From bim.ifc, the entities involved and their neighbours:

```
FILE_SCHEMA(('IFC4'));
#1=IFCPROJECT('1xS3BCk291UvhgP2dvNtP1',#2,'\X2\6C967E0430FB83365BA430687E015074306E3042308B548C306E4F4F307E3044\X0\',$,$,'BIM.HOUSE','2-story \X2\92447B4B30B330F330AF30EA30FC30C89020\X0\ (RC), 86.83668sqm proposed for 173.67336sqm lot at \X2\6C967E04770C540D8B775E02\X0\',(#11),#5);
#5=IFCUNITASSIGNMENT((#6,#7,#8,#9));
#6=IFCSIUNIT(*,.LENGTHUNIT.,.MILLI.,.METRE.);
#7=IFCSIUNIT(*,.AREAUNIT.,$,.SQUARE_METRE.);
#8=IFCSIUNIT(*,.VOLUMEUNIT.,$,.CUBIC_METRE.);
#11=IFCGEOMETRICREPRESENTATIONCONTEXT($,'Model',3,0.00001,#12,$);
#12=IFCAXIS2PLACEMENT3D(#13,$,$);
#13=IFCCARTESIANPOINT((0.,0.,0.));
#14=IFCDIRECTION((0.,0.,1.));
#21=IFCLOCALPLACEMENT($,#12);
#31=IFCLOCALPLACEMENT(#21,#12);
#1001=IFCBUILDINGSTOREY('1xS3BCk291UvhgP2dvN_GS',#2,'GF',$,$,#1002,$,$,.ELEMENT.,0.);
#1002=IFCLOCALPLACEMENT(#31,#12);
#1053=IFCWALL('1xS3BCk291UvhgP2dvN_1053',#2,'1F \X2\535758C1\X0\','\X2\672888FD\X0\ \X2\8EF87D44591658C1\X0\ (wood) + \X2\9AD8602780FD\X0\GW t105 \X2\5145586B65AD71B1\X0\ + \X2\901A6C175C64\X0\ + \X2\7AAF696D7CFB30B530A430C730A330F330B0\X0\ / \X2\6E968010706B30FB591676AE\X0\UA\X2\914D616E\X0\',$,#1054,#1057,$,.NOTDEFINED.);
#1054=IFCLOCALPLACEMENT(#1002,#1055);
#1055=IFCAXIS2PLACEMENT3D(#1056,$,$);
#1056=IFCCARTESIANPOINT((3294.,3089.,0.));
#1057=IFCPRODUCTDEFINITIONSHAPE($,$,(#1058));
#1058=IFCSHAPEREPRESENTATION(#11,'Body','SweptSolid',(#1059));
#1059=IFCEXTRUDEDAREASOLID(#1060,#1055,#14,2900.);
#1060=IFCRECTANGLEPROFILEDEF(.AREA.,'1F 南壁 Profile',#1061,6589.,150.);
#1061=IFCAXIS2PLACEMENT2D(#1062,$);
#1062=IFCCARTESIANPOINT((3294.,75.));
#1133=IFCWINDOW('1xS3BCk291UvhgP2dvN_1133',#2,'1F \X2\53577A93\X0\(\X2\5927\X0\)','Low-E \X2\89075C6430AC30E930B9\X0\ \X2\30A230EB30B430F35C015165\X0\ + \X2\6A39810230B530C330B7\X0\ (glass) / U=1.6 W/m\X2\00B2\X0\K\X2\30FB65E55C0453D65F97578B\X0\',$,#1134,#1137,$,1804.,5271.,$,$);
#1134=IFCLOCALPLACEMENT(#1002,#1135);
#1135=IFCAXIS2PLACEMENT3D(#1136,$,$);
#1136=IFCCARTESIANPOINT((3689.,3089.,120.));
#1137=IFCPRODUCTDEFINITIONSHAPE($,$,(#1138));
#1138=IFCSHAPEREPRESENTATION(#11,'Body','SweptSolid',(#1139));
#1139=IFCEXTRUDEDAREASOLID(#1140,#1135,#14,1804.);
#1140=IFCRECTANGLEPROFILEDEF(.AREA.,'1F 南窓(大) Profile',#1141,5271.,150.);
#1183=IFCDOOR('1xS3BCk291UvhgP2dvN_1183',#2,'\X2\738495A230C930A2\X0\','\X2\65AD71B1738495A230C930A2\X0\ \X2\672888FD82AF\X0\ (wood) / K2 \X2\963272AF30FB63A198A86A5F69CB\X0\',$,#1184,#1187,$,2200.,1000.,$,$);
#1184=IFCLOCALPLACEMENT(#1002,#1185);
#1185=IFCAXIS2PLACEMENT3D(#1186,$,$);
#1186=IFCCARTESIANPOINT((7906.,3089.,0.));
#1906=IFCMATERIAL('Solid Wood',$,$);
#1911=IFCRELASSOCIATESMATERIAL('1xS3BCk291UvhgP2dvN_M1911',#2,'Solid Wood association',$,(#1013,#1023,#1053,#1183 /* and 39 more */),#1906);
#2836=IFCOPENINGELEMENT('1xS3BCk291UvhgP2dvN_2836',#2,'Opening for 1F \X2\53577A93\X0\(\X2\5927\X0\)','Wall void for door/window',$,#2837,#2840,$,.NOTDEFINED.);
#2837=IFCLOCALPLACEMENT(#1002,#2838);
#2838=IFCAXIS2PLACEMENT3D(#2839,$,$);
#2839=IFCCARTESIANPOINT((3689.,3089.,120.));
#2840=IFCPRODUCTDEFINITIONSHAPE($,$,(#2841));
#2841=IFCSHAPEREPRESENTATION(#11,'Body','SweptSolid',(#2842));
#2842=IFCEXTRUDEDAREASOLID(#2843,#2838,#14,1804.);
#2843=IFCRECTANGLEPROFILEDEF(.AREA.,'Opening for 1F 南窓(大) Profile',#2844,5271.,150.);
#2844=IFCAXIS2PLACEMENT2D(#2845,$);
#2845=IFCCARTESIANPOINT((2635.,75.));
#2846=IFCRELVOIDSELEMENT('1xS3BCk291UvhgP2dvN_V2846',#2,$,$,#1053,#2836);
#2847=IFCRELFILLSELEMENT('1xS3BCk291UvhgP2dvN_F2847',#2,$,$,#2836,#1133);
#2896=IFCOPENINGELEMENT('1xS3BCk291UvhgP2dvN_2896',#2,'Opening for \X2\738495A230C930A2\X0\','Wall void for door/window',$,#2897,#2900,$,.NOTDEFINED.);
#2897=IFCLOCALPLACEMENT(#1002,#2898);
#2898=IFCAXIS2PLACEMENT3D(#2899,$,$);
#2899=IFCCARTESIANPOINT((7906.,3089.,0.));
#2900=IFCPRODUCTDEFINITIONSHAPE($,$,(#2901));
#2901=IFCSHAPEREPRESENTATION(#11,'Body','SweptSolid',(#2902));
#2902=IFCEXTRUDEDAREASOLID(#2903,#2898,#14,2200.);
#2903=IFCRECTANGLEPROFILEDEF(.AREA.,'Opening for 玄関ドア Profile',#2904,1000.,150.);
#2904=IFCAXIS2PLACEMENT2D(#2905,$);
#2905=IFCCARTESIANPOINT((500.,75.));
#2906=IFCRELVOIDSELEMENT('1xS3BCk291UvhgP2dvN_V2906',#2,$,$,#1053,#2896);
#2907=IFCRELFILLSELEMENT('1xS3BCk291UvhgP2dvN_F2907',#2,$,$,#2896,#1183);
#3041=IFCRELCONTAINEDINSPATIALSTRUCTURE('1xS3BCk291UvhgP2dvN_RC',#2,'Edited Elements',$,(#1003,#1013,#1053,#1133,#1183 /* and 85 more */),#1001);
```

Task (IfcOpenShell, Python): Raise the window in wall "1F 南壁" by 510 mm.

```python
import numpy as np
import ifcopenshell
import ifcopenshell.api.geometry
import ifcopenshell.util.placement
import ifcopenshell.util.unit

model = ifcopenshell.open("bim.ifc")
unit_scale = ifcopenshell.util.unit.calculate_unit_scale(model)

window = model.by_guid("1xS3BCk291UvhgP2dvN_1133")
opening = window.FillsVoids[0].RelatingOpeningElement
dz = 510.0

shift = np.array([0.0, 0.0, dz])
# The window is not placed relative to its opening, so move both.
for product in (opening, window):
    matrix = ifcopenshell.util.placement.get_local_placement(product.ObjectPlacement)
    matrix[:3, 3] += shift
    ifcopenshell.api.geometry.edit_object_placement(model, product=product, matrix=matrix, is_si=False)

print(f"moved by {dz * unit_scale:+.3f} m")

model.write("bim_edited.ifc")
```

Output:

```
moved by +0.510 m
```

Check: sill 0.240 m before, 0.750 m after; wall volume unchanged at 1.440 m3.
